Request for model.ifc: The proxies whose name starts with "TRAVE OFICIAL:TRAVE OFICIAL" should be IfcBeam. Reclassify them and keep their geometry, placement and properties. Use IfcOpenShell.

First a look at what the model holds.

```python
import re

import ifcopenshell

model = ifcopenshell.open("model.ifc")
print(model.schema)
seen = {}
for e in model.by_type("IfcBuildingElementProxy"):
    name = re.sub(r":\d+(:\d+)?$", "", e.Name or "")  # drop the element id that some exporters append
    seen[name] = seen.get(name, 0) + 1
for name, count in sorted(seen.items()):
    print(count, "x", name)
```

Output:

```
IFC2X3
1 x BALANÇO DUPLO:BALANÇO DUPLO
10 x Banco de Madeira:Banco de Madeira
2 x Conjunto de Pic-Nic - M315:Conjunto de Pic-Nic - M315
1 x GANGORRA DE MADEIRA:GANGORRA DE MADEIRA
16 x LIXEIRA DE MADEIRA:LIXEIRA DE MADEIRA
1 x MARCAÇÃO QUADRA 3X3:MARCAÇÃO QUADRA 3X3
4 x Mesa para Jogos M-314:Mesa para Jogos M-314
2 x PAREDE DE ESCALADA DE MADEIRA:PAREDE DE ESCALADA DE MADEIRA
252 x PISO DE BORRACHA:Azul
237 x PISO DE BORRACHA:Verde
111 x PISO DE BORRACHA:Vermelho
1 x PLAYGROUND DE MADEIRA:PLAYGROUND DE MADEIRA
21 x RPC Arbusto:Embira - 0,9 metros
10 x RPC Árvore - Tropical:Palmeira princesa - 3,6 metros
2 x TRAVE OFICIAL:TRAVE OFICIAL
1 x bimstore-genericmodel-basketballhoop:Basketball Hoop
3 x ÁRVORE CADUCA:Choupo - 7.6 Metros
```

```python
import ifcopenshell
import ifcopenshell.api.root

model = ifcopenshell.open("model.ifc")

proxies = [e.id() for e in model.by_type("IfcBuildingElementProxy") if (e.Name or "").startswith("TRAVE OFICIAL:TRAVE OFICIAL")]
for step_id in proxies:
    proxy = model.by_id(step_id)
    # Reclassifying a typed element also reclassifies its type and the type's other occurrences.
    if proxy.is_a("IfcBuildingElementProxy"):
        ifcopenshell.api.root.reassign_class(model, product=proxy, ifc_class="IfcBeam")

print(sum(model.by_id(i).is_a("IfcBeam") for i in proxies), "reclassified")

model.write("model_rev.ifc")
```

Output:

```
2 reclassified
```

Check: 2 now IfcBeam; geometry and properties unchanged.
